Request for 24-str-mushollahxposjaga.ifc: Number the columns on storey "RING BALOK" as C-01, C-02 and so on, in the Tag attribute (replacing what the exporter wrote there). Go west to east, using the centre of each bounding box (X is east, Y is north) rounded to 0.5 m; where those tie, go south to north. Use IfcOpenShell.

First a look at what the model holds.

```python
import ifcopenshell
import ifcopenshell.util.element
import ifcopenshell.util.placement

model = ifcopenshell.open("24-str-mushollahxposjaga.ifc")
print(model.schema)
storey = next(s for s in model.by_type("IfcBuildingStorey") if s.Name == "RING BALOK")
columns = [e for e in ifcopenshell.util.element.get_decomposition(storey) if e.is_a("IfcColumn")]
for e in sorted(columns, key=lambda e: e.id()):
    origin = ifcopenshell.util.placement.get_local_placement(e.ObjectPlacement)[:3, 3]
    print(e.id(), e.Tag, e.Name, origin.round(2) + 0.0, sep=" | ")
```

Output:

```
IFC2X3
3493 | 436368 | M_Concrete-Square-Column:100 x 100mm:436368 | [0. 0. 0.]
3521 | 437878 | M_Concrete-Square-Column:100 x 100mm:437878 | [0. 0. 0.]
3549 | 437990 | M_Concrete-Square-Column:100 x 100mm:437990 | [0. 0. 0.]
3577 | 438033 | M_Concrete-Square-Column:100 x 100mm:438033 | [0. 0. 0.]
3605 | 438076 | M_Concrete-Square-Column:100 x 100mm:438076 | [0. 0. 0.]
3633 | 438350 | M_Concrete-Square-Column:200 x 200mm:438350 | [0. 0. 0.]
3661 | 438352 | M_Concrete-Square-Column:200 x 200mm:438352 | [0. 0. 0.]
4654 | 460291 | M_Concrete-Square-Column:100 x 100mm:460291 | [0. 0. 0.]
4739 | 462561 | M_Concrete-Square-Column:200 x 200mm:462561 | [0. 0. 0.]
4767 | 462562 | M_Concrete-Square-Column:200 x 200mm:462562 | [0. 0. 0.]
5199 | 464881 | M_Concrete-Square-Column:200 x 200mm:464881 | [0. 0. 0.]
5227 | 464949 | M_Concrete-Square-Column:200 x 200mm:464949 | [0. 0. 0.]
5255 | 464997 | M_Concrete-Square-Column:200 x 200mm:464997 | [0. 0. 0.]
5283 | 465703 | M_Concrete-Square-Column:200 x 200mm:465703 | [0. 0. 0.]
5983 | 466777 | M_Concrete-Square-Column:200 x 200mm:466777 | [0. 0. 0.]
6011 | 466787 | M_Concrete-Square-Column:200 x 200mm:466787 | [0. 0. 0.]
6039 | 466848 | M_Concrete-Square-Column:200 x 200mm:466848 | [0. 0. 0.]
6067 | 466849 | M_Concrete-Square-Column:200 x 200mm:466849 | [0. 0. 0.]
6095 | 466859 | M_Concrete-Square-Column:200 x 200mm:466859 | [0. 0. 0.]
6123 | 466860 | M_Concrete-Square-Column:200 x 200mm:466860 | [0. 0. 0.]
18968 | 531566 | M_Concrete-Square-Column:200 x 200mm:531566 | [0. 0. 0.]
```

```python
import ifcopenshell
import ifcopenshell.geom
import ifcopenshell.util.element
import ifcopenshell.util.shape

model = ifcopenshell.open("24-str-mushollahxposjaga.ifc")
settings = ifcopenshell.geom.settings()
settings.set("use-world-coords", True)


def centre(element):
    shape = ifcopenshell.geom.create_shape(settings, element)
    return ifcopenshell.util.shape.get_bbox_centroid(shape.geometry)


storey = next(s for s in model.by_type("IfcBuildingStorey") if s.Name == "RING BALOK")
columns = [e for e in ifcopenshell.util.element.get_decomposition(storey) if e.is_a("IfcColumn")]

# Insertion points can sit at a corner or the storey origin, so sort by the geometry (in metres).
centres = {e: centre(e) for e in columns}
columns.sort(key=lambda e: (round(centres[e][0] / 0.5), centres[e][1]))

for i, e in enumerate(columns, start=1):
    number = f"C-{i:02d}"
    e.Tag = number
    print(e.id(), number)

model.write("24-str-mushollahxposjaga_updated.ifc")
```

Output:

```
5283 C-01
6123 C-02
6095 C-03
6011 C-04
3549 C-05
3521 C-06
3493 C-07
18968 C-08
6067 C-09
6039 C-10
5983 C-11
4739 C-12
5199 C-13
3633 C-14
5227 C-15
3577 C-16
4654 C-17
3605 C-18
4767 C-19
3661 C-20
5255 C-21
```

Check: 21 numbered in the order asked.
